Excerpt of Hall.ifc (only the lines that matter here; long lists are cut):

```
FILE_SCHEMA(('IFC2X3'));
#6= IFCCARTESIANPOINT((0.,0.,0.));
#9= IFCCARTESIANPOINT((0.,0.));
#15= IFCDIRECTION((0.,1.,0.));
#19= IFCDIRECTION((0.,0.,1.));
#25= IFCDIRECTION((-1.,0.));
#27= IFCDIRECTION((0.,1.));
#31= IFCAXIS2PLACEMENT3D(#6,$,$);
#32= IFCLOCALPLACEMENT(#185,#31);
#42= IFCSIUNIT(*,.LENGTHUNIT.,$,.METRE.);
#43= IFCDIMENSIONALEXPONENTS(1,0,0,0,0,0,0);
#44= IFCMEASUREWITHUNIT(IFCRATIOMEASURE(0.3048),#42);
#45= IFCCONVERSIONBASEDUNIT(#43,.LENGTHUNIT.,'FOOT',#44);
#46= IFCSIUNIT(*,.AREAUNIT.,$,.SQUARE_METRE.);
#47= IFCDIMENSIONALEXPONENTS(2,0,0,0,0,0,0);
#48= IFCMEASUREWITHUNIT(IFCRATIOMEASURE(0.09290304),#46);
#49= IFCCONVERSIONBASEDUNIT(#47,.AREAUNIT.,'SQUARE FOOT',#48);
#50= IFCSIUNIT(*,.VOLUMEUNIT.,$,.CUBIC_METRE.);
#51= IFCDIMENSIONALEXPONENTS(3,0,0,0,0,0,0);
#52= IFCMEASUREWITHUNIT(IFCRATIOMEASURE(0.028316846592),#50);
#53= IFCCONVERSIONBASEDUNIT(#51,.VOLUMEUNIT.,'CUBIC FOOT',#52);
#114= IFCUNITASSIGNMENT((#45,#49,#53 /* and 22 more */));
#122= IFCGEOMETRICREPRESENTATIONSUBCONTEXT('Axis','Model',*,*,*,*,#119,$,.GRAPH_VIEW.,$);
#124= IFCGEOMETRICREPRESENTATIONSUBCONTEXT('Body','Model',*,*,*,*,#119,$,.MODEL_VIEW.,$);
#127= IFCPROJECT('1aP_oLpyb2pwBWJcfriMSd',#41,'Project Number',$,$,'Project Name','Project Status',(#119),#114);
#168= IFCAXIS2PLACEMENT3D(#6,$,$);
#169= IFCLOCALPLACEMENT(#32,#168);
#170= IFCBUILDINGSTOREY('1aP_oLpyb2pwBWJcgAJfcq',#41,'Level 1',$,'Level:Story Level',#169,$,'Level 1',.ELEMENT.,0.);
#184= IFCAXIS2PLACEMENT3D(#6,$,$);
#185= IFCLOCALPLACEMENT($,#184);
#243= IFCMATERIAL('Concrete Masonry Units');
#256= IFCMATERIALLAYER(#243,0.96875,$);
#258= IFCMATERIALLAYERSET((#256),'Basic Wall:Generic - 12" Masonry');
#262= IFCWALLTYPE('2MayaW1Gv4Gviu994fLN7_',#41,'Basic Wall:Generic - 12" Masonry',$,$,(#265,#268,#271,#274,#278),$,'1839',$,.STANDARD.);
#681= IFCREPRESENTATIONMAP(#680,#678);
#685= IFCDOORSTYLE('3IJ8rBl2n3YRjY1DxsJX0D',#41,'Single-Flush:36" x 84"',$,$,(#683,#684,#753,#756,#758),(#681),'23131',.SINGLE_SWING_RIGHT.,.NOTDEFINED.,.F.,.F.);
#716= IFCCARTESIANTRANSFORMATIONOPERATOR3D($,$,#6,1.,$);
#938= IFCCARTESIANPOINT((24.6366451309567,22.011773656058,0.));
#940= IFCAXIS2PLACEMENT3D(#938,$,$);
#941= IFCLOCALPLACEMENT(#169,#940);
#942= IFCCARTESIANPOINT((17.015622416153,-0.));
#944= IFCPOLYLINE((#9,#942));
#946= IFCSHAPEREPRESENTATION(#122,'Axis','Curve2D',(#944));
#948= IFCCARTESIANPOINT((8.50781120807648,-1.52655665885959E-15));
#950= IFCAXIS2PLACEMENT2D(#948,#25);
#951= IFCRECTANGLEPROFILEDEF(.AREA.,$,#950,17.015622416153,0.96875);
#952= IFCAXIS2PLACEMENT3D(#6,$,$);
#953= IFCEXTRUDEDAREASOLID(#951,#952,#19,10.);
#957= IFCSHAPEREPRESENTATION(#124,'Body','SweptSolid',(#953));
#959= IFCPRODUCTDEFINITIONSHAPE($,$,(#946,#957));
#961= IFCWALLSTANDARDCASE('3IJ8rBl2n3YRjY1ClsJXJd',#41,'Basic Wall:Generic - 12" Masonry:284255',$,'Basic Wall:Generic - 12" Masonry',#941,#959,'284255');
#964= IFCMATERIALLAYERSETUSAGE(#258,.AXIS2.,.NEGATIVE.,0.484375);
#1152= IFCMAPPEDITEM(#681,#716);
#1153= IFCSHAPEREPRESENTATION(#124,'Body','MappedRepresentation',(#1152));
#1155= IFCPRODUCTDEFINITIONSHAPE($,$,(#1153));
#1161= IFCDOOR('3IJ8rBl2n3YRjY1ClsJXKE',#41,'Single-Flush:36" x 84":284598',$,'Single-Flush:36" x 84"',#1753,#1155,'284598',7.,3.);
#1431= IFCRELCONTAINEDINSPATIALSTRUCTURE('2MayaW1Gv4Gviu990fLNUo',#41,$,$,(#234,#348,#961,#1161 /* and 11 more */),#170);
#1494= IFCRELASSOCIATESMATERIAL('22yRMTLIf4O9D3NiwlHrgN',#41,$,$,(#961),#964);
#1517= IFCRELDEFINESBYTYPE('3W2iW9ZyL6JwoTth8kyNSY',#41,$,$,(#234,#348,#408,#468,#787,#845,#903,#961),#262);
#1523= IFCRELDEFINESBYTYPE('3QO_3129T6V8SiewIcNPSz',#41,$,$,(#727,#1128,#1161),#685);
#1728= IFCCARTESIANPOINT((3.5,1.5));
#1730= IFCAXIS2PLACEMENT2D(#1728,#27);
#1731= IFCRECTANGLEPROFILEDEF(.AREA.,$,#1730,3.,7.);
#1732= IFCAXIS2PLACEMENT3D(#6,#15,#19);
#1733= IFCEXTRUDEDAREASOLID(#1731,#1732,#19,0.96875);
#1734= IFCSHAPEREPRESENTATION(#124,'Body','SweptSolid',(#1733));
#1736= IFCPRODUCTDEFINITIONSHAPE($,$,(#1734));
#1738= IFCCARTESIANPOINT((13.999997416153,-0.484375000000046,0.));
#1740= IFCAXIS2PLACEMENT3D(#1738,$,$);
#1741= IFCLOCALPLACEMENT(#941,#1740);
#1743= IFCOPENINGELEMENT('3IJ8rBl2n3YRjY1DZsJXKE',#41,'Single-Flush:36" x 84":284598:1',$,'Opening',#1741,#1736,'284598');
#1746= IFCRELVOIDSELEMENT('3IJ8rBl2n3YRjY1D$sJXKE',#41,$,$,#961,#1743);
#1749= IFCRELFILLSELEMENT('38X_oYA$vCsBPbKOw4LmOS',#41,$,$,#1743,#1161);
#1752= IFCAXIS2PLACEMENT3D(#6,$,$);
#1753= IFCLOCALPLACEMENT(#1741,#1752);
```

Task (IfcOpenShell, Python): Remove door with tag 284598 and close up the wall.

```python
import ifcopenshell
import ifcopenshell.api.feature
import ifcopenshell.api.root
import ifcopenshell.geom
import ifcopenshell.util.shape

model = ifcopenshell.open("Hall.ifc")
settings = ifcopenshell.geom.settings()


def volume(element):
    """Net volume in cubic metres, openings subtracted."""
    shape = ifcopenshell.geom.create_shape(settings, element)
    return ifcopenshell.util.shape.get_volume(shape.geometry)


door = model.by_guid("3IJ8rBl2n3YRjY1ClsJXKE")
opening = door.FillsVoids[0].RelatingOpeningElement
wall = opening.VoidsElements[0].RelatingBuildingElement
before = volume(wall)

ifcopenshell.api.root.remove_product(model, product=door)
ifcopenshell.api.feature.remove_feature(model, feature=opening)

after = volume(wall)

print(f"wall volume {before:.3f} -> {after:.3f} m3")

model.write("Hall_v2.ifc")
```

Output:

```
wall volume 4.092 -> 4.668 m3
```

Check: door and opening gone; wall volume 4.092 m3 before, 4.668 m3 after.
